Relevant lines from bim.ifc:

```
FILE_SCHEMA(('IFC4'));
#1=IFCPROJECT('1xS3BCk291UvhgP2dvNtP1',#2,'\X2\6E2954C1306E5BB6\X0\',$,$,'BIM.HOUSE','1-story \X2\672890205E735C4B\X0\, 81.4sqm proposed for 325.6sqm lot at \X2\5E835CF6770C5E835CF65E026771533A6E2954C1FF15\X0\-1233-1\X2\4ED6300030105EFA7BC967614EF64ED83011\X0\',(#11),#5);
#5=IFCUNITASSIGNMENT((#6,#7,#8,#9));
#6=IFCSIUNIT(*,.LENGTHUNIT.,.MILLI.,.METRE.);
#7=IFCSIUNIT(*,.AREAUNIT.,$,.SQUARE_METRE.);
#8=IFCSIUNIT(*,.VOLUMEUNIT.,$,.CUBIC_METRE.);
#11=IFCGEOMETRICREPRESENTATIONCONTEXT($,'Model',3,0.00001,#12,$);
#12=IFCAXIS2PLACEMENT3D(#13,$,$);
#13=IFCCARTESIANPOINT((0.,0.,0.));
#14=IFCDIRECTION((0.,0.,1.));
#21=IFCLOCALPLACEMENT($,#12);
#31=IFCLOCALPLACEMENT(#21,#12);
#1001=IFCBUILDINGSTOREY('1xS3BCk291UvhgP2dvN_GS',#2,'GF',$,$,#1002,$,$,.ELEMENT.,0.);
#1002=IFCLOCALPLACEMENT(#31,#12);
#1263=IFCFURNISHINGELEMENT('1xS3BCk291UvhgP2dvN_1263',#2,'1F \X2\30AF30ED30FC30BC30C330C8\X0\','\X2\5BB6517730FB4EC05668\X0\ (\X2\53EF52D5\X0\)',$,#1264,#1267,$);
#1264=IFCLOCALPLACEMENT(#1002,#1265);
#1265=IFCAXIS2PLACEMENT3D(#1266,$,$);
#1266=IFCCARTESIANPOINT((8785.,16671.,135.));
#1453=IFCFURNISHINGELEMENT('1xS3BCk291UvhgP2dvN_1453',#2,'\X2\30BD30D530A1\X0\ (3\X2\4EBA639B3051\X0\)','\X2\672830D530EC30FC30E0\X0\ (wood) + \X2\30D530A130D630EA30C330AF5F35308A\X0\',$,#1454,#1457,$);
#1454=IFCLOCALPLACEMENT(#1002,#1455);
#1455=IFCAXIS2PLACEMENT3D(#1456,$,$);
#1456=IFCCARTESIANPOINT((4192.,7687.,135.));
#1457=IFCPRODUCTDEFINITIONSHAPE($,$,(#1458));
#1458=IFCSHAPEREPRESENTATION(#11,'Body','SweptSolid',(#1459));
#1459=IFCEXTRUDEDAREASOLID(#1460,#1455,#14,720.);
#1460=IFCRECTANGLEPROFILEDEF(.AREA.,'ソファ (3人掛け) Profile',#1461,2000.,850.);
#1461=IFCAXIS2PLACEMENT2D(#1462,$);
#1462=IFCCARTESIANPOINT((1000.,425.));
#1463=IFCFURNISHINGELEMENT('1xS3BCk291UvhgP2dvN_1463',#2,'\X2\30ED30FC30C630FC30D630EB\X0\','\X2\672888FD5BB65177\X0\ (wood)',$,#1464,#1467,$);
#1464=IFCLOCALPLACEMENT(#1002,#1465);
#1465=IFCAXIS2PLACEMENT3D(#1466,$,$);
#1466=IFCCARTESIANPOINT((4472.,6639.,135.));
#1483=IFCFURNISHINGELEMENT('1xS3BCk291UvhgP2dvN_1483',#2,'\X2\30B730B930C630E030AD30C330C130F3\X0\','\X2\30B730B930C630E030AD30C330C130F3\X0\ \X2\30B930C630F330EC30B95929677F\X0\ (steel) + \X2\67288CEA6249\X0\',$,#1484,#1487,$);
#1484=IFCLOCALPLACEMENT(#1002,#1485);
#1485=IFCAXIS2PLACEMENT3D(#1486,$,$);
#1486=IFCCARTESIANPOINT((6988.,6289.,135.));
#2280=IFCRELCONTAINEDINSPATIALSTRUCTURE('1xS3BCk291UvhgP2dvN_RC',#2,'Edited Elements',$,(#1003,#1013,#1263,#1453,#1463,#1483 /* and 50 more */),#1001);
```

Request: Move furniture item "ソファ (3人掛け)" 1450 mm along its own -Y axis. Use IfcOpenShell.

```python
import ifcopenshell
import ifcopenshell.api.geometry
import ifcopenshell.util.placement
import ifcopenshell.util.unit

model = ifcopenshell.open("bim.ifc")
unit_scale = ifcopenshell.util.unit.calculate_unit_scale(model)

item = model.by_guid("1xS3BCk291UvhgP2dvN_1453")
matrix = ifcopenshell.util.placement.get_local_placement(item.ObjectPlacement)
matrix[:3, 3] -= matrix[:3, 1] * 1.45 / unit_scale
ifcopenshell.api.geometry.edit_object_placement(model, product=item, matrix=matrix, is_si=False)

print(ifcopenshell.util.placement.get_local_placement(item.ObjectPlacement).round(3) + 0.0)

model.write("bim_edited.ifc")
```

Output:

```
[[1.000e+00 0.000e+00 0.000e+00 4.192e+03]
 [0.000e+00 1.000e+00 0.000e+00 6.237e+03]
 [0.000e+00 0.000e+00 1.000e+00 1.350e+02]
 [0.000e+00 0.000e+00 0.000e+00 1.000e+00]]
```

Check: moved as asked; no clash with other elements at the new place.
